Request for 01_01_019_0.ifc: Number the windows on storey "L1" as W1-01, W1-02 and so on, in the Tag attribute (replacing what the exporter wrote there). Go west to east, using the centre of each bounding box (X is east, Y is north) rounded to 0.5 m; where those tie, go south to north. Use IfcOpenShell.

First a look at what the model holds.

```python
import ifcopenshell
import ifcopenshell.util.element
import ifcopenshell.util.placement

model = ifcopenshell.open("01_01_019_0.ifc")
print(model.schema)
storey = next(s for s in model.by_type("IfcBuildingStorey") if s.Name == "L1")
windows = [e for e in ifcopenshell.util.element.get_decomposition(storey) if e.is_a("IfcWindow")]
for e in sorted(windows, key=lambda e: e.id()):
    origin = ifcopenshell.util.placement.get_local_placement(e.ObjectPlacement)[:3, 3]
    print(e.id(), e.Tag, e.Name, origin.round(2) + 0.0, sep=" | ")
```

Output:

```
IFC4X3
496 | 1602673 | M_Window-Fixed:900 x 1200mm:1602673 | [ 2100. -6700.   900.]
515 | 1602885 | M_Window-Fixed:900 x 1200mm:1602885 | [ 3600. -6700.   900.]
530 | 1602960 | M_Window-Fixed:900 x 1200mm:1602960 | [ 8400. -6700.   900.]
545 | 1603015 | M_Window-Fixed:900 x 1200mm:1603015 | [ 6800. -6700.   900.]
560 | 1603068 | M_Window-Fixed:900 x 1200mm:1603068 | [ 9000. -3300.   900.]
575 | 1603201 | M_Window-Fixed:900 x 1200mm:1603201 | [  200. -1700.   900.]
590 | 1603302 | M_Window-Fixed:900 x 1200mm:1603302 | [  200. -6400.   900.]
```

```python
import ifcopenshell
import ifcopenshell.geom
import ifcopenshell.util.element
import ifcopenshell.util.shape

model = ifcopenshell.open("01_01_019_0.ifc")
settings = ifcopenshell.geom.settings()
settings.set("use-world-coords", True)


def centre(element):
    shape = ifcopenshell.geom.create_shape(settings, element)
    return ifcopenshell.util.shape.get_bbox_centroid(shape.geometry)


storey = next(s for s in model.by_type("IfcBuildingStorey") if s.Name == "L1")
windows = [e for e in ifcopenshell.util.element.get_decomposition(storey) if e.is_a("IfcWindow")]

# Insertion points can sit at a corner or the storey origin, so sort by the geometry (in metres).
centres = {e: centre(e) for e in windows}
windows.sort(key=lambda e: (round(centres[e][0] / 0.5), centres[e][1]))

for i, e in enumerate(windows, start=1):
    number = f"W1-{i:02d}"
    e.Tag = number
    print(e.id(), number)

model.write("01_01_019_0_v2.ifc")
```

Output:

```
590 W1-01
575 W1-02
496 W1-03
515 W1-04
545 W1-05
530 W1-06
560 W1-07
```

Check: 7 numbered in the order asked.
